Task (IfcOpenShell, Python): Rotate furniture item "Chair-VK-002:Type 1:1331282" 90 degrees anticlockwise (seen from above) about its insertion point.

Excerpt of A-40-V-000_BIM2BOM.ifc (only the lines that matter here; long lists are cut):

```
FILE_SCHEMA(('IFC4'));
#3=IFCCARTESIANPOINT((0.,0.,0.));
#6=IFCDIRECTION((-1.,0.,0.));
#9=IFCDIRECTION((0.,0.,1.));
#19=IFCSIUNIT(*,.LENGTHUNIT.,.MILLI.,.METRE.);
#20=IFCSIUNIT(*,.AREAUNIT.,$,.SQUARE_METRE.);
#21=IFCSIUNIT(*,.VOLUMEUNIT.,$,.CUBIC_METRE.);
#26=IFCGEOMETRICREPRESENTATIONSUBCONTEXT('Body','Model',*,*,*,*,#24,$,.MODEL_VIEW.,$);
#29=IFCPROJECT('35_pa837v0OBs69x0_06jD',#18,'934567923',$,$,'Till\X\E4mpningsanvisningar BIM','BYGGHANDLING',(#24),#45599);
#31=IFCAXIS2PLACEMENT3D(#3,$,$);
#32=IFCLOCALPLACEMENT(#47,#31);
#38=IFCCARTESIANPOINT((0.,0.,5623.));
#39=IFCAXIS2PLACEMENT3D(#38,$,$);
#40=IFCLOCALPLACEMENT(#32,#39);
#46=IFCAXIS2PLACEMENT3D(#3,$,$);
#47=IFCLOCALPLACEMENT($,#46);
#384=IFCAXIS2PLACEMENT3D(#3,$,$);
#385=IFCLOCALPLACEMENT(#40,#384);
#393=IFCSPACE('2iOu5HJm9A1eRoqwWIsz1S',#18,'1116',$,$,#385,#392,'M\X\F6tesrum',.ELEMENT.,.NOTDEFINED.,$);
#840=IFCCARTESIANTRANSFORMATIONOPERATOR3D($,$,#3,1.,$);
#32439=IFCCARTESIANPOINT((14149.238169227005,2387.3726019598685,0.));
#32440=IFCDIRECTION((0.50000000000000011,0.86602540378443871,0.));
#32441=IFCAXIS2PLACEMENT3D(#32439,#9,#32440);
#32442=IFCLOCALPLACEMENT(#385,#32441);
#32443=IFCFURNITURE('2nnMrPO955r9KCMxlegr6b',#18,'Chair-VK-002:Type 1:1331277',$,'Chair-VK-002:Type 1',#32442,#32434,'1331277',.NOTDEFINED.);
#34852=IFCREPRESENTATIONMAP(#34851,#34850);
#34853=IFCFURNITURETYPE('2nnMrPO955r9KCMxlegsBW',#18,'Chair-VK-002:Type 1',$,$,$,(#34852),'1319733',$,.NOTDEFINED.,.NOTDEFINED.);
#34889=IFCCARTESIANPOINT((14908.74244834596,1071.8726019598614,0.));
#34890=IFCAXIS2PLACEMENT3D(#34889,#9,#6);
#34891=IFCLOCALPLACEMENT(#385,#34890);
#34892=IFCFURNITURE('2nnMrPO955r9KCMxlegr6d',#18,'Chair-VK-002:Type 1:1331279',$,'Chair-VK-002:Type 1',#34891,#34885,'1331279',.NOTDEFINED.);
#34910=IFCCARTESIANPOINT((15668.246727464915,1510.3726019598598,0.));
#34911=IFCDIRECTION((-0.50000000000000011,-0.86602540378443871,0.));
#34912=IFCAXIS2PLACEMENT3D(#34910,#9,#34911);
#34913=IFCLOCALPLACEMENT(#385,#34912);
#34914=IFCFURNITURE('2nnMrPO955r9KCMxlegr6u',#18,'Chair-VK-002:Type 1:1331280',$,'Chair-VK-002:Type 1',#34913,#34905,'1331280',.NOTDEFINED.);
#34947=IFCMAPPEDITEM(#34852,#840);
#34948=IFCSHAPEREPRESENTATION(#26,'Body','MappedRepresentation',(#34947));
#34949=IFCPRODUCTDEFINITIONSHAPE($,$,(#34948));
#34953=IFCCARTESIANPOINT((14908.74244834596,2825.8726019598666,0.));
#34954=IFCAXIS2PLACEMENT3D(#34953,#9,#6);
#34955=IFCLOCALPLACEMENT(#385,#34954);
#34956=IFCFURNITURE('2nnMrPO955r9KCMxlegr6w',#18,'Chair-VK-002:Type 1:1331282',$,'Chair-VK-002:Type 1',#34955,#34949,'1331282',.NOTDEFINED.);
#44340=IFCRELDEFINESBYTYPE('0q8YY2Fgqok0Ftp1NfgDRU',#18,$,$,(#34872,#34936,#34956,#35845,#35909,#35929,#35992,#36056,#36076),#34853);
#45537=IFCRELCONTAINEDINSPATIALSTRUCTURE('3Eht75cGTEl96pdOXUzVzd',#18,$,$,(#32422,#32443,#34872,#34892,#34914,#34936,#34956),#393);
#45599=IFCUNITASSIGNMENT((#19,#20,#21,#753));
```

```python
import ifcopenshell
import ifcopenshell.api.geometry
import ifcopenshell.util.placement

model = ifcopenshell.open("A-40-V-000_BIM2BOM.ifc")

item = model.by_guid("2nnMrPO955r9KCMxlegr6w")
matrix = ifcopenshell.util.placement.get_local_placement(item.ObjectPlacement)
matrix = matrix @ ifcopenshell.util.placement.rotation(90, "Z")
ifcopenshell.api.geometry.edit_object_placement(model, product=item, matrix=matrix, is_si=False)

print(ifcopenshell.util.placement.get_local_placement(item.ObjectPlacement).round(3) + 0.0)

model.write("A-40-V-000_BIM2BOM_v2.ifc")
```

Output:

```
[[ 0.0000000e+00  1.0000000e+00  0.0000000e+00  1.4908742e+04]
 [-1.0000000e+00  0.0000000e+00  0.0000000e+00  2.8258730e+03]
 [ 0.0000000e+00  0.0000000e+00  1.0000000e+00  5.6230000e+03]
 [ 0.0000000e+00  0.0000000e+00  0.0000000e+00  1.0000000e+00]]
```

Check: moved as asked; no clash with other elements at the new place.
